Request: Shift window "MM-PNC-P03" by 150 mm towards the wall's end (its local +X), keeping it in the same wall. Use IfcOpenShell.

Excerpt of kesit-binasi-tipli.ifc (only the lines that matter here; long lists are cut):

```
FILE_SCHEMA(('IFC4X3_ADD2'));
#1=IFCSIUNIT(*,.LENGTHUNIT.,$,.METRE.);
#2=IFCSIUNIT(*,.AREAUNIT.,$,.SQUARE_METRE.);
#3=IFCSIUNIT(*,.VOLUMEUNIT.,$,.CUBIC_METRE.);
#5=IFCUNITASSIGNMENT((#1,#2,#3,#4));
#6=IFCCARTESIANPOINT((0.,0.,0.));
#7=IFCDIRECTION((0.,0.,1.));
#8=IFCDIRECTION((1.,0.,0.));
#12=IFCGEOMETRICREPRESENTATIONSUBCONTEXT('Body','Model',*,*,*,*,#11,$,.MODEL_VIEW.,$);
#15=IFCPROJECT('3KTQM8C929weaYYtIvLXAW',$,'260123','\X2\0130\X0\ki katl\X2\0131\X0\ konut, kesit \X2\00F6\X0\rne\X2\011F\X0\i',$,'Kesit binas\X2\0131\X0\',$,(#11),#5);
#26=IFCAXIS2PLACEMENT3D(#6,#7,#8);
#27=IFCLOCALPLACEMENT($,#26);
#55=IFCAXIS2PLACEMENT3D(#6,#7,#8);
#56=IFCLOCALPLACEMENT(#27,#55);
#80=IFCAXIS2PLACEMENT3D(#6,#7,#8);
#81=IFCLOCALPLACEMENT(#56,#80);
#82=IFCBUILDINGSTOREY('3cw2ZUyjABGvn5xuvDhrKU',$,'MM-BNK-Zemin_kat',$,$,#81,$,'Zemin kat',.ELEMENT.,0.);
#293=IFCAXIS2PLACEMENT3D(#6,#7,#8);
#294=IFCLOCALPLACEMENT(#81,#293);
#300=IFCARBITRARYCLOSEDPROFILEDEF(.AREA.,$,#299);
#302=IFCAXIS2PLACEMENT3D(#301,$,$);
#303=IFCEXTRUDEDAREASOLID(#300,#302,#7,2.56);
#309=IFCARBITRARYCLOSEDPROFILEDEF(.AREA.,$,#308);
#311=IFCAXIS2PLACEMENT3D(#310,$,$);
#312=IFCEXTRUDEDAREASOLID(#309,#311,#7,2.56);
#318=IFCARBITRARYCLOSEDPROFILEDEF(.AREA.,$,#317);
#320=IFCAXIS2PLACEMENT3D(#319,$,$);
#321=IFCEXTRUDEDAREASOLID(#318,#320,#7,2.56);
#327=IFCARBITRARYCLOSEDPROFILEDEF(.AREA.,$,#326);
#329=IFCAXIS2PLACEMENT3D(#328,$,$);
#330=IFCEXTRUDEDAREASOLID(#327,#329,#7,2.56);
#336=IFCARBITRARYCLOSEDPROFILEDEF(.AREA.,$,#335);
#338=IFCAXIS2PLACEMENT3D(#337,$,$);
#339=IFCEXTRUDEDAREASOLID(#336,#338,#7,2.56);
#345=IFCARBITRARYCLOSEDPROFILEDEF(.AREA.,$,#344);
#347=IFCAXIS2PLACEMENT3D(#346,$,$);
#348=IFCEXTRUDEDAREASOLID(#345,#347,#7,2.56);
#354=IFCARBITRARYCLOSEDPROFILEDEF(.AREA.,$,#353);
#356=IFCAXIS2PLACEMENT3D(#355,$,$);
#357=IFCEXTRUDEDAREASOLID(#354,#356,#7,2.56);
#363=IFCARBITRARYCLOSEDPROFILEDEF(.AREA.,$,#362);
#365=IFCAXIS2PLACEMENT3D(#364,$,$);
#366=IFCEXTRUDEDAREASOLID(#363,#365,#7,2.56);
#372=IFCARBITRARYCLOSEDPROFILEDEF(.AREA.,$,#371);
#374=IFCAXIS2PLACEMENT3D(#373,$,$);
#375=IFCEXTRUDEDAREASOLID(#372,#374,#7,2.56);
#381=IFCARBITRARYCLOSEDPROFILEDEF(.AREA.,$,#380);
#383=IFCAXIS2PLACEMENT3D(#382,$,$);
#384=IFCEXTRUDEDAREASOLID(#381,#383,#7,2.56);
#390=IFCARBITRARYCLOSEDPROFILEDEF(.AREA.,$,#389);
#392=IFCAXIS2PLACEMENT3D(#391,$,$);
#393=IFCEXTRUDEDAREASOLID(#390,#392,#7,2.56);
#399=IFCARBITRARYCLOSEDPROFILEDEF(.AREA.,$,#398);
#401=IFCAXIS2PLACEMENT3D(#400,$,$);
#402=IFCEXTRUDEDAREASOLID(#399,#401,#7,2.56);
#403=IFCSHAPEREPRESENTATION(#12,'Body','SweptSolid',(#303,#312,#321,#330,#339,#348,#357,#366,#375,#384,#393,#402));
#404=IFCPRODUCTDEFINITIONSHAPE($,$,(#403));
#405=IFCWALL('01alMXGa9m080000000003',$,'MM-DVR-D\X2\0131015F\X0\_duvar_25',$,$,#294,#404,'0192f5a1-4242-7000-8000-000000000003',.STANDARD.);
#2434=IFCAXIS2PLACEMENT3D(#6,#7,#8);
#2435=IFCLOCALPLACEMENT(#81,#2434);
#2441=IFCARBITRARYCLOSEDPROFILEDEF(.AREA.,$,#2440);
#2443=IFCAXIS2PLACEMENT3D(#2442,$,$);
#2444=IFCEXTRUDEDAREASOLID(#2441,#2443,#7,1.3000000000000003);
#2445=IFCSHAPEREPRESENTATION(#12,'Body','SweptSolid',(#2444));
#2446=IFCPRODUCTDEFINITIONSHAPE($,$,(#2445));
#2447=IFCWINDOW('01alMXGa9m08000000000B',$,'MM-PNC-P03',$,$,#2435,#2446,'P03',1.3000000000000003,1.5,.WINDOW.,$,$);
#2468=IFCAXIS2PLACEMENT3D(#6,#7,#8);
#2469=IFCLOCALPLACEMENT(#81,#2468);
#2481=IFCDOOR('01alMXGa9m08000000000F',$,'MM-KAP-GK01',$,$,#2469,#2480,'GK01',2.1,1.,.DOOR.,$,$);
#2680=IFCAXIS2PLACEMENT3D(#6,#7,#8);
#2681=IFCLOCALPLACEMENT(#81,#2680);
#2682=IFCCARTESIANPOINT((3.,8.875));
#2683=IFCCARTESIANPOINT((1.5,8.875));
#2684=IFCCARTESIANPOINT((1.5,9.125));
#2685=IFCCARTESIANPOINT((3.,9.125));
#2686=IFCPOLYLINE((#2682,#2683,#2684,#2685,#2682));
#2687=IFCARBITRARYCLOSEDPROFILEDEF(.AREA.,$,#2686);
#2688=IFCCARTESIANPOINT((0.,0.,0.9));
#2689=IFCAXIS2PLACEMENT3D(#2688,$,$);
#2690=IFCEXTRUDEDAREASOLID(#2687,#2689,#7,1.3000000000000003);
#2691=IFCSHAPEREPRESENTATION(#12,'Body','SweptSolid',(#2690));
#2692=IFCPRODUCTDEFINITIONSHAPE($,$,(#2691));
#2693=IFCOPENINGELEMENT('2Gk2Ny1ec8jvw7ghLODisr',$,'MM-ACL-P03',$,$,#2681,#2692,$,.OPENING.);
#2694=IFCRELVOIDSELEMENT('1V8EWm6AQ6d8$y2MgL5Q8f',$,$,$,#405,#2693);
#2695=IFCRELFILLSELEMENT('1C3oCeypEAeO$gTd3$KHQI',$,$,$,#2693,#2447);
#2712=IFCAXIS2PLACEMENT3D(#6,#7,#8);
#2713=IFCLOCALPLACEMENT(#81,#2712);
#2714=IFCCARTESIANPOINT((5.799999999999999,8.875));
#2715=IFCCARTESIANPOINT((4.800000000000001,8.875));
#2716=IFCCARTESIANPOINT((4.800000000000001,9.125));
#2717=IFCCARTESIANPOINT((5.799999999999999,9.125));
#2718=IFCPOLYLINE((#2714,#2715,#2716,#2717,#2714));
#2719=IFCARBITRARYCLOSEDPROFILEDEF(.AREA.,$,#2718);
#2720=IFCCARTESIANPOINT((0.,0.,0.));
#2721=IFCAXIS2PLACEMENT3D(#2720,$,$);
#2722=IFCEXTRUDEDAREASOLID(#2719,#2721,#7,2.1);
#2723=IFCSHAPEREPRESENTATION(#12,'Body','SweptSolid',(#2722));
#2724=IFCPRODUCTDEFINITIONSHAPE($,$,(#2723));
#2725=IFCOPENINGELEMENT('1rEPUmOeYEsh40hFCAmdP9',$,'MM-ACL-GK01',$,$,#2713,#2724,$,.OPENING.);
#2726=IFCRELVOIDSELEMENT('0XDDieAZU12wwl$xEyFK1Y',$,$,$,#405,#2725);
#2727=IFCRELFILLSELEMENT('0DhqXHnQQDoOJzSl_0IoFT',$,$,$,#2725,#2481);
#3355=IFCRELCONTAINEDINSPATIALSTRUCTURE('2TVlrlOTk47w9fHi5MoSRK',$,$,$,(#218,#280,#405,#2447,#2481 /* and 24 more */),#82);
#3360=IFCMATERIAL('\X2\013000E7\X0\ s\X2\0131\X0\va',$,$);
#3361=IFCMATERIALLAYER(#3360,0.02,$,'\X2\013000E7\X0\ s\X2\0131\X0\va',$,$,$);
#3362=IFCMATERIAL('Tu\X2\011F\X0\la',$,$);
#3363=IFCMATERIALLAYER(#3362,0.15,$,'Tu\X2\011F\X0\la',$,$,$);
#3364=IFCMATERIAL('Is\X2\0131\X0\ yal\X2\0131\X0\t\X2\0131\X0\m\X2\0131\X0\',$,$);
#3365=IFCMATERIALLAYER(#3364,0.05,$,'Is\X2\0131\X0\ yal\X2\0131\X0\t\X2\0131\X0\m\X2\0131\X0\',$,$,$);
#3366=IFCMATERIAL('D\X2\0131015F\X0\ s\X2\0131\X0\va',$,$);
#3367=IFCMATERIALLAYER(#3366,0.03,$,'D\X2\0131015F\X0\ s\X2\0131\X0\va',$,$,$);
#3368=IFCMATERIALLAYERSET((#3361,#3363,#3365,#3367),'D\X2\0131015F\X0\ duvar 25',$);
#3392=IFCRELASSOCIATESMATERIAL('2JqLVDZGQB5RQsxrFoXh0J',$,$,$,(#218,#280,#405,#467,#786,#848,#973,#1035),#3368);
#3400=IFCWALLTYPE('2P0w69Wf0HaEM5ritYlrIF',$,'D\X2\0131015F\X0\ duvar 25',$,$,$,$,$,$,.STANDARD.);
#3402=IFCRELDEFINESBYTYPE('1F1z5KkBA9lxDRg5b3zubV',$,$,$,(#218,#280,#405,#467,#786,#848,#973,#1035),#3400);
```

```python
import ifcopenshell
import ifcopenshell.api.geometry
import ifcopenshell.util.placement
import ifcopenshell.util.unit

model = ifcopenshell.open("kesit-binasi-tipli.ifc")
unit_scale = ifcopenshell.util.unit.calculate_unit_scale(model)

window = model.by_id(2447)
opening = window.FillsVoids[0].RelatingOpeningElement
wall = opening.VoidsElements[0].RelatingBuildingElement

wall_matrix = ifcopenshell.util.placement.get_local_placement(wall.ObjectPlacement)
shift = wall_matrix[:3, 0] * 0.15 / unit_scale
before = ifcopenshell.util.placement.get_local_placement(window.ObjectPlacement)[:3, 3].copy()

# The window is not placed relative to its opening, so move both.
for product in (opening, window):
    matrix = ifcopenshell.util.placement.get_local_placement(product.ObjectPlacement)
    matrix[:3, 3] += shift
    ifcopenshell.api.geometry.edit_object_placement(model, product=product, matrix=matrix, is_si=False)

after = ifcopenshell.util.placement.get_local_placement(window.ObjectPlacement)[:3, 3]
print("window moved by", (after - before).round(3) + 0.0)

model.write("kesit-binasi-tipli_v2.ifc")
```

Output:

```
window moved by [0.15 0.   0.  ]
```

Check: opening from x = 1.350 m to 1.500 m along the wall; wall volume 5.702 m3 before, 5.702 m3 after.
